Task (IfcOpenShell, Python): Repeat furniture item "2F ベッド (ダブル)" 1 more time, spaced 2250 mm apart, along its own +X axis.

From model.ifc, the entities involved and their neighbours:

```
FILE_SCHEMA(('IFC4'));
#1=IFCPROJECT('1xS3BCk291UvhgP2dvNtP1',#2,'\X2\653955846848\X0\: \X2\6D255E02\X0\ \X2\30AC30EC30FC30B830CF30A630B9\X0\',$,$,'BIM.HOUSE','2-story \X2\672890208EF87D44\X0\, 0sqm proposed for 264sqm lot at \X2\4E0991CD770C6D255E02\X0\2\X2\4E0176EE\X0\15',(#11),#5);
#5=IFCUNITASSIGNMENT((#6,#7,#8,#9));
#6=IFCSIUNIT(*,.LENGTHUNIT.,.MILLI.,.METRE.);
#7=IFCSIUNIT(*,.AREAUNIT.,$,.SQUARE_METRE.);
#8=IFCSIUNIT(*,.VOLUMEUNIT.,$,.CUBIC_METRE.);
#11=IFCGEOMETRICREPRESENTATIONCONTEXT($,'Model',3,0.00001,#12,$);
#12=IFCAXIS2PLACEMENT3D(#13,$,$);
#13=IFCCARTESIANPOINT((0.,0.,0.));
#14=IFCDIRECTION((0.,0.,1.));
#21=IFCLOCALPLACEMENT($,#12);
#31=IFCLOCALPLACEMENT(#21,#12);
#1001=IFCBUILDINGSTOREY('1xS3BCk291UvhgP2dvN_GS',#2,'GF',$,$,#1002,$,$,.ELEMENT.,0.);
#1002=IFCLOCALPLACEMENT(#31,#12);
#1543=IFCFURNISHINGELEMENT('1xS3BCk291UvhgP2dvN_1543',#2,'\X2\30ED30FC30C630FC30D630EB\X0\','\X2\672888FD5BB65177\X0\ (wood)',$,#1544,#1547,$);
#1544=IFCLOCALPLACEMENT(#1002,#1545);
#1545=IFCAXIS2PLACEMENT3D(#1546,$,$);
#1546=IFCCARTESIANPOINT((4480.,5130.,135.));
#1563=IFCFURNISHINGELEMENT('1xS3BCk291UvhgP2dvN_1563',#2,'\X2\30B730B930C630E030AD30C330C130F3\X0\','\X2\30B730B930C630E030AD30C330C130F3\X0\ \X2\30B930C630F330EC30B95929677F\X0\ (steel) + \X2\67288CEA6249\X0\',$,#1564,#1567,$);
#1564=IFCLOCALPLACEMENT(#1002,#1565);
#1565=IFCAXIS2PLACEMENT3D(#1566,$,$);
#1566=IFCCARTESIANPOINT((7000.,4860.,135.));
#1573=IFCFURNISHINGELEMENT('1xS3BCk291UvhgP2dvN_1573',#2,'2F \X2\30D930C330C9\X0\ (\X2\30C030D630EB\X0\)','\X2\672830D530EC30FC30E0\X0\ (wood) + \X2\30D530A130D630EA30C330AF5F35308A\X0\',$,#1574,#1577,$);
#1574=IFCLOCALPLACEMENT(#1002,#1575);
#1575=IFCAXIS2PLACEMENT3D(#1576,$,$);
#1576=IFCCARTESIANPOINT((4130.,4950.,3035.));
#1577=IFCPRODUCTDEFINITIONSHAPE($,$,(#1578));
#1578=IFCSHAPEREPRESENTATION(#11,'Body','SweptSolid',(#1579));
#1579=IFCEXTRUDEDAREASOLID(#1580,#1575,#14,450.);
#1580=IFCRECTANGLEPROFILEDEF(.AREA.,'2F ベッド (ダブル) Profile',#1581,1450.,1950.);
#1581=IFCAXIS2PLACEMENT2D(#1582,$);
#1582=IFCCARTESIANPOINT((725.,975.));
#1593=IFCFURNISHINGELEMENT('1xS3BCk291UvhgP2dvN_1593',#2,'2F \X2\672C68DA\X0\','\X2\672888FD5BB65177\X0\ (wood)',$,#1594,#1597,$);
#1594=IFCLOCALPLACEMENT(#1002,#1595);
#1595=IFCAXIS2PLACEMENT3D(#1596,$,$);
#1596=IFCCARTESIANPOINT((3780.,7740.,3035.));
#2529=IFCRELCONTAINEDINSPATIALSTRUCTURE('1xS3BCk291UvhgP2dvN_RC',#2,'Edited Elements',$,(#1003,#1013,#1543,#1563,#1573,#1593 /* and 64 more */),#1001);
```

```python
import ifcopenshell
import ifcopenshell.api.geometry
import ifcopenshell.api.root
import ifcopenshell.util.element
import ifcopenshell.util.placement
import ifcopenshell.util.unit

model = ifcopenshell.open("model.ifc")
unit_scale = ifcopenshell.util.unit.calculate_unit_scale(model)


def reuse_history(source, copy):
    """copy_class also copies each property set's owner history, people and application; keep the originals."""
    for rel in copy.IsDefinedBy:
        if rel.is_a("IfcRelDefinesByProperties") and (history := rel.RelatingPropertyDefinition.OwnerHistory):
            rel.RelatingPropertyDefinition.OwnerHistory = source.OwnerHistory
            ifcopenshell.util.element.remove_deep2(model, history)


source = model.by_guid("1xS3BCk291UvhgP2dvN_1573")
base = ifcopenshell.util.placement.get_local_placement(source.ObjectPlacement)
step = base[:3, 0] * 2.25 / unit_scale

for i in range(1, 2):
    copy = ifcopenshell.api.root.copy_class(model, product=source)
    copy.Representation = ifcopenshell.util.element.copy_deep(
        model, source.Representation, exclude=["IfcGeometricRepresentationContext", "IfcRepresentationMap"]
    )
    reuse_history(source, copy)
    matrix = base.copy()
    matrix[:3, 3] += i * step
    print("added at", matrix[:3, 3].round(3) + 0.0)
    ifcopenshell.api.geometry.edit_object_placement(model, product=copy, matrix=matrix, is_si=False)

model.write("model_edited.ifc")
```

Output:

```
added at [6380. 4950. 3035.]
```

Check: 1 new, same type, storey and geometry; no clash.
